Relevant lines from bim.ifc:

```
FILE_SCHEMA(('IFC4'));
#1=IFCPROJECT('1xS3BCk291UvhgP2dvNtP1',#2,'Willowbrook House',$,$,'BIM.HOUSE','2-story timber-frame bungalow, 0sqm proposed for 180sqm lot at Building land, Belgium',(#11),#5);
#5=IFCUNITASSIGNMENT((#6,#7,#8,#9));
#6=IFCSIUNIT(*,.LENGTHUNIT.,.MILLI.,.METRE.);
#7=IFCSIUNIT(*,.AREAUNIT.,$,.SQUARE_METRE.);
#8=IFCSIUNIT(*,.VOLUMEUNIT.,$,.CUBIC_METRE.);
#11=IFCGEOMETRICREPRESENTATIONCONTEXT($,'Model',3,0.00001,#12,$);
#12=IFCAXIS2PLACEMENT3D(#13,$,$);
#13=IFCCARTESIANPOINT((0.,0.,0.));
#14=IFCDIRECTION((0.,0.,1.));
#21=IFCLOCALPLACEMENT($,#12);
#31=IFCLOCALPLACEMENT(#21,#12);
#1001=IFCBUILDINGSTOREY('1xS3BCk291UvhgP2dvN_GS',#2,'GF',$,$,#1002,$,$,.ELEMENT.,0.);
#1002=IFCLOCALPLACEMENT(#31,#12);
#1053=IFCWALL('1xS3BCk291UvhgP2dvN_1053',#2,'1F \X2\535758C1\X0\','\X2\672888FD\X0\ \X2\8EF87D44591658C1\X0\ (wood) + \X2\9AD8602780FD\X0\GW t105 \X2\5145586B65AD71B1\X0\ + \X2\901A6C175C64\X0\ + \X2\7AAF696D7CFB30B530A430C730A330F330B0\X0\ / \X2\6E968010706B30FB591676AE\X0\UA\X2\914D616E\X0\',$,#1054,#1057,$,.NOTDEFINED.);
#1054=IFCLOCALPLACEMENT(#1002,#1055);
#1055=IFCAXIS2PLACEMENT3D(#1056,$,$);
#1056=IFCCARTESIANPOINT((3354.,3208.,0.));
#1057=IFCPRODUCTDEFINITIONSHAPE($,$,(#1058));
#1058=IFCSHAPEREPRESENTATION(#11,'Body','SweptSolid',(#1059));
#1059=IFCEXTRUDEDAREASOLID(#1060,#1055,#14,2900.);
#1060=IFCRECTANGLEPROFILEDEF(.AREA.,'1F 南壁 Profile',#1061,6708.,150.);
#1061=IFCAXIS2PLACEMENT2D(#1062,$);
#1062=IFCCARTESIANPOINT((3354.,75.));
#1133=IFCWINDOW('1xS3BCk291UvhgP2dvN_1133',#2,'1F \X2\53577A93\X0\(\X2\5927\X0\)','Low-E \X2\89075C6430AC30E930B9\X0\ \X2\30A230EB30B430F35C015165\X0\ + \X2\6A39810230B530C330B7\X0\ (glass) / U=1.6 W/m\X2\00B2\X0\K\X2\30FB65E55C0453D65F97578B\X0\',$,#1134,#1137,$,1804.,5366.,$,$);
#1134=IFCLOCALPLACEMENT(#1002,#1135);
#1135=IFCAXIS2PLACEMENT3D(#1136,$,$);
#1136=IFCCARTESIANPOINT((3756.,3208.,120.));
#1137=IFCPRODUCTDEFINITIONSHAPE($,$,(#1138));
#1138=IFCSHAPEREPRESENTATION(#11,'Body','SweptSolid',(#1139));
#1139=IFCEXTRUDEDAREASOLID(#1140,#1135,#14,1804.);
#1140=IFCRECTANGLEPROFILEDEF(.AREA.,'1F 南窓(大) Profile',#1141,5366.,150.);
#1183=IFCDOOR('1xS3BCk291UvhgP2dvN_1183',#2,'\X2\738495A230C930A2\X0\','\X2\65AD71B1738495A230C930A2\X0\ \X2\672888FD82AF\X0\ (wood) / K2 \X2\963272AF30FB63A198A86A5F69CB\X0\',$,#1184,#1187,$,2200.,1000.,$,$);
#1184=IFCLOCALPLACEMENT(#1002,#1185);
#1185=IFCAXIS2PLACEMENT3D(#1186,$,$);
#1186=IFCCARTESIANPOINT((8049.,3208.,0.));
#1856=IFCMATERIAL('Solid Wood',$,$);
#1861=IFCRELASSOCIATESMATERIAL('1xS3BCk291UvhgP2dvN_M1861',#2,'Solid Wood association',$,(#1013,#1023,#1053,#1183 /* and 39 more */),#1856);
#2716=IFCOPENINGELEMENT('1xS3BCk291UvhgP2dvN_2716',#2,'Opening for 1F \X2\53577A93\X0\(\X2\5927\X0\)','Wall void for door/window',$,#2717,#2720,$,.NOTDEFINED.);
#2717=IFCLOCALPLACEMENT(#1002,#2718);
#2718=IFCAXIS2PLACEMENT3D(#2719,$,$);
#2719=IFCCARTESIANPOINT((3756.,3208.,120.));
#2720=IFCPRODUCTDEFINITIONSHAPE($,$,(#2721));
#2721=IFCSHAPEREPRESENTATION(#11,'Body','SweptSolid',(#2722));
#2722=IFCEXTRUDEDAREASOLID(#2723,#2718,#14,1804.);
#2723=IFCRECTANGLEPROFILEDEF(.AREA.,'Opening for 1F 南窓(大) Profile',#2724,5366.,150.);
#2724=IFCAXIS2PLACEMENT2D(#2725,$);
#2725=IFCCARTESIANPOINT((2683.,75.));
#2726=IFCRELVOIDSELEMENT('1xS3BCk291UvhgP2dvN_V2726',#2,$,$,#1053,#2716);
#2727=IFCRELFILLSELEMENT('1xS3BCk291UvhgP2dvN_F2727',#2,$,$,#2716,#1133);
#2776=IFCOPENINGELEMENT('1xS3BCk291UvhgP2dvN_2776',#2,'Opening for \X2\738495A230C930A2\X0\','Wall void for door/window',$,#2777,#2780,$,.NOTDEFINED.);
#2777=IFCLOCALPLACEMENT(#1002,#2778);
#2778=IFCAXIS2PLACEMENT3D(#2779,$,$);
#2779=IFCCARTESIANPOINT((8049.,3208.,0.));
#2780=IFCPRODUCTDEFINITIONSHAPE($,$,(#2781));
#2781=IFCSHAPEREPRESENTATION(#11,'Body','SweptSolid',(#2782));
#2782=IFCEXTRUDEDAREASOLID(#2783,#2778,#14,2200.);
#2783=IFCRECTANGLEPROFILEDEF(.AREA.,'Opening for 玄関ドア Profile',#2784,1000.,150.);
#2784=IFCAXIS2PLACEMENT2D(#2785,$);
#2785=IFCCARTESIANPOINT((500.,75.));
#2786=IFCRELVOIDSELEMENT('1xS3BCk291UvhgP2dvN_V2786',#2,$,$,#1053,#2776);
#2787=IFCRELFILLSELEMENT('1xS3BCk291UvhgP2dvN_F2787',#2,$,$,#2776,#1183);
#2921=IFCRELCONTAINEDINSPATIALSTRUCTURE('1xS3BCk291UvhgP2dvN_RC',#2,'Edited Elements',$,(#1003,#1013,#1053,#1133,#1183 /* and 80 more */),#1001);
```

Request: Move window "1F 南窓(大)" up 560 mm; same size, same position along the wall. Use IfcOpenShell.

```python
import numpy as np
import ifcopenshell
import ifcopenshell.api.geometry
import ifcopenshell.util.placement
import ifcopenshell.util.unit

model = ifcopenshell.open("bim.ifc")
unit_scale = ifcopenshell.util.unit.calculate_unit_scale(model)

window = model.by_guid("1xS3BCk291UvhgP2dvN_1133")
opening = window.FillsVoids[0].RelatingOpeningElement
dz = 0.56 / unit_scale

shift = np.array([0.0, 0.0, dz])
# The window is not placed relative to its opening, so move both.
for product in (opening, window):
    matrix = ifcopenshell.util.placement.get_local_placement(product.ObjectPlacement)
    matrix[:3, 3] += shift
    ifcopenshell.api.geometry.edit_object_placement(model, product=product, matrix=matrix, is_si=False)

print(f"moved by {dz * unit_scale:+.3f} m")

model.write("bim_edited.ifc")
```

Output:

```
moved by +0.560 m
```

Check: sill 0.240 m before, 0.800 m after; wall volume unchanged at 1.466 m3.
